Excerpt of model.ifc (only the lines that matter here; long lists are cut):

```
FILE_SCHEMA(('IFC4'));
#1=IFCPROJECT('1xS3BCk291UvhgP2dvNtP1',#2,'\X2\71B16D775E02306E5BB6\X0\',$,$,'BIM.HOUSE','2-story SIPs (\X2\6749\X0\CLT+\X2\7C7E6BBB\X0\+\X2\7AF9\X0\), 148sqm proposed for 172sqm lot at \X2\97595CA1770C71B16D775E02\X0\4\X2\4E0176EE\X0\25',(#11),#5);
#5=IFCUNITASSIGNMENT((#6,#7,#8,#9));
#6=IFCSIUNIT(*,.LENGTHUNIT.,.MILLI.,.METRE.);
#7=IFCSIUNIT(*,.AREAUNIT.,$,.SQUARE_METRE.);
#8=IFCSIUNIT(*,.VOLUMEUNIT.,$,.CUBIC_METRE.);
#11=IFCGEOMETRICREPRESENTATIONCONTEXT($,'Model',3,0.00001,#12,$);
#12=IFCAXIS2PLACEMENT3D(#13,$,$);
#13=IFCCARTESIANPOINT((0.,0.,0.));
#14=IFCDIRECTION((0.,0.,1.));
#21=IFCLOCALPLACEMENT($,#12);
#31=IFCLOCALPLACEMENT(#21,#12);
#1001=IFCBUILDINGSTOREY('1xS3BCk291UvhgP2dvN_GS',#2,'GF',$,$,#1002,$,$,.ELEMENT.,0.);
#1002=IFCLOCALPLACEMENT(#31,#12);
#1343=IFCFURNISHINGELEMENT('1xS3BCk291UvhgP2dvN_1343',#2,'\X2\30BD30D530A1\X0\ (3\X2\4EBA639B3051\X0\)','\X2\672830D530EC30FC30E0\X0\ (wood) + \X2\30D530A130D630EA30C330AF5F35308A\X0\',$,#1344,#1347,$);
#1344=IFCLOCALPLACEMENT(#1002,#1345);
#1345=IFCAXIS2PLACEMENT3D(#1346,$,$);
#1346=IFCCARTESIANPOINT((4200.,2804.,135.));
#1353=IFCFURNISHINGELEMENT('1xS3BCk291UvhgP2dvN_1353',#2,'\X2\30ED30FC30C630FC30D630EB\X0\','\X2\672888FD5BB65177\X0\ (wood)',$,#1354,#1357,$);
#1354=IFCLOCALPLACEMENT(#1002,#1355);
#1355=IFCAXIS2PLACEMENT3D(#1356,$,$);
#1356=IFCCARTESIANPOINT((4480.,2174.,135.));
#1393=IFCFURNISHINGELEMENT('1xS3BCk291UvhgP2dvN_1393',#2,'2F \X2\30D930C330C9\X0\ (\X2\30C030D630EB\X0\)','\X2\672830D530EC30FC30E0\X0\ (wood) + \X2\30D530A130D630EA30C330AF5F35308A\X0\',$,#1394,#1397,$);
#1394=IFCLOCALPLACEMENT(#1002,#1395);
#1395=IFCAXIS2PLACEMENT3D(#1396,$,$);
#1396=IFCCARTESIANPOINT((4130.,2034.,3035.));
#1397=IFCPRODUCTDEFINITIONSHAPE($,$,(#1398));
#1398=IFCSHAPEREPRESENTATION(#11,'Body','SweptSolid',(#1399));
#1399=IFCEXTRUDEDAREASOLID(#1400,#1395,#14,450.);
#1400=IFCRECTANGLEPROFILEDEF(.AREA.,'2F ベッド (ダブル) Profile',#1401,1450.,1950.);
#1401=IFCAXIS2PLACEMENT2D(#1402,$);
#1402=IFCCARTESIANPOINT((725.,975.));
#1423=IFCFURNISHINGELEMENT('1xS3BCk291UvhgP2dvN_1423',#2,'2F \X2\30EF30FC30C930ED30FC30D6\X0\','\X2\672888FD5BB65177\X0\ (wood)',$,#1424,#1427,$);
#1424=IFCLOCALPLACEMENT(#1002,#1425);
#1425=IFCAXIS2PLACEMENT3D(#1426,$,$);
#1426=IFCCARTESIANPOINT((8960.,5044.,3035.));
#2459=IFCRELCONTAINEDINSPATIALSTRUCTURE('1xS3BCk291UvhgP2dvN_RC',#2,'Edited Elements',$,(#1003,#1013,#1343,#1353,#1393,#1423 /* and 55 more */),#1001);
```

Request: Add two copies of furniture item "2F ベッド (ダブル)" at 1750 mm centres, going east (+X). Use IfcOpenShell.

```python
import numpy as np
import ifcopenshell
import ifcopenshell.api.geometry
import ifcopenshell.api.root
import ifcopenshell.util.element
import ifcopenshell.util.placement
import ifcopenshell.util.unit

model = ifcopenshell.open("model.ifc")
unit_scale = ifcopenshell.util.unit.calculate_unit_scale(model)


def reuse_history(source, copy):
    """copy_class also copies each property set's owner history, people and application; keep the originals."""
    for rel in copy.IsDefinedBy:
        if rel.is_a("IfcRelDefinesByProperties") and (history := rel.RelatingPropertyDefinition.OwnerHistory):
            rel.RelatingPropertyDefinition.OwnerHistory = source.OwnerHistory
            ifcopenshell.util.element.remove_deep2(model, history)


source = model.by_guid("1xS3BCk291UvhgP2dvN_1393")
base = ifcopenshell.util.placement.get_local_placement(source.ObjectPlacement)
step = np.array([1.0, 0.0, 0.0]) * 1.75 / unit_scale

for i in range(1, 3):
    copy = ifcopenshell.api.root.copy_class(model, product=source)
    copy.Representation = ifcopenshell.util.element.copy_deep(
        model, source.Representation, exclude=["IfcGeometricRepresentationContext", "IfcRepresentationMap"]
    )
    reuse_history(source, copy)
    matrix = base.copy()
    matrix[:3, 3] += i * step
    print("added at", matrix[:3, 3].round(3) + 0.0)
    ifcopenshell.api.geometry.edit_object_placement(model, product=copy, matrix=matrix, is_si=False)

model.write("model-out.ifc")
```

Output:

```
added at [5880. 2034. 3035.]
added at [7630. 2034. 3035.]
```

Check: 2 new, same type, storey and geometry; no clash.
